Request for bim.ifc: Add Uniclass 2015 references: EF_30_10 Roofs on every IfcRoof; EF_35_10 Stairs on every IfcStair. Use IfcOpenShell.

First a look at what the model holds.

```python
import ifcopenshell

model = ifcopenshell.open("bim.ifc")
print(model.schema)
print("classifications:", [c.Name for c in model.by_type("IfcClassification")])
for ifc_class in ("IfcDoor", "IfcRoof", "IfcStair", "IfcWall", "IfcWindow"):
    print(ifc_class, len(model.by_type(ifc_class)))
```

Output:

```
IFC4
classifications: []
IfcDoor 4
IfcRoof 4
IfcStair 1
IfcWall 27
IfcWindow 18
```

```python
import ifcopenshell
import ifcopenshell.api.classification

model = ifcopenshell.open("bim.ifc")

system = ifcopenshell.api.classification.add_classification(model, classification="Uniclass 2015")

codes = {
    "IfcRoof": ("EF_30_10", "Roofs"),
    "IfcStair": ("EF_35_10", "Stairs"),
}
for ifc_class, (code, name) in codes.items():
    products = model.by_type(ifc_class)
    ifcopenshell.api.classification.add_reference(
        model, products=products, classification=system, identification=code, name=name
    )
    print(code, len(products))

model.write("bim_edited.ifc")
```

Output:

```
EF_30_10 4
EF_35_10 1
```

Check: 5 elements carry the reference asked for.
